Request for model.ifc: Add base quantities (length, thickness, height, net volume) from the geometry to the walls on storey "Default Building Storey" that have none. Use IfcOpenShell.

First a look at what the model holds.

```python
import ifcopenshell
import ifcopenshell.util.element
import ifcopenshell.util.unit

model = ifcopenshell.open("model.ifc")
print(model.schema)
for unit_type in ("LENGTHUNIT", "AREAUNIT", "VOLUMEUNIT"):
    print(unit_type, ifcopenshell.util.unit.calculate_unit_scale(model, unit_type))
storey = next(s for s in model.by_type("IfcBuildingStorey") if s.Name == "Default Building Storey")
walls = [e for e in ifcopenshell.util.element.get_decomposition(storey) if e.is_a("IfcWall")]
for e in sorted(walls, key=lambda e: e.id()):
    print(e.id(), e.is_a(), e.Name, list(ifcopenshell.util.element.get_psets(e, qtos_only=True)), sep=" | ")
```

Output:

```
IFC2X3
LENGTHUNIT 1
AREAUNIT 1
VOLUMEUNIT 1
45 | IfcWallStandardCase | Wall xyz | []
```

```python
import ifcopenshell
import ifcopenshell.api.pset
import ifcopenshell.geom
import ifcopenshell.util.element
import ifcopenshell.util.shape
import ifcopenshell.util.unit

model = ifcopenshell.open("model.ifc")
unit_scale = ifcopenshell.util.unit.calculate_unit_scale(model)
volume_scale = ifcopenshell.util.unit.calculate_unit_scale(model, "VOLUMEUNIT")
settings = ifcopenshell.geom.settings()

storey = next(s for s in model.by_type("IfcBuildingStorey") if s.Name == "Default Building Storey")
walls = [e for e in ifcopenshell.util.element.get_decomposition(storey) if e.is_a("IfcWall")]

for e in sorted(walls, key=lambda e: e.id()):
    if ifcopenshell.util.element.get_psets(e, qtos_only=True, should_inherit=False):
        continue
    # Geometry comes back in metres, in the element's own axes.
    shape = ifcopenshell.geom.create_shape(settings, e)
    values = {
        "Length": ifcopenshell.util.shape.get_x(shape.geometry) / unit_scale,
        "Width": ifcopenshell.util.shape.get_y(shape.geometry) / unit_scale,
        "Height": ifcopenshell.util.shape.get_z(shape.geometry) / unit_scale,
        "NetVolume": ifcopenshell.util.shape.get_volume(shape.geometry) / volume_scale,
    }
    qto = ifcopenshell.api.pset.add_qto(model, product=e, name="BaseQuantities")
    ifcopenshell.api.pset.edit_qto(model, qto=qto, properties=values)
    print(e.id(), {k: round(v, 3) for k, v in values.items()})

model.write("model_edited.ifc")
```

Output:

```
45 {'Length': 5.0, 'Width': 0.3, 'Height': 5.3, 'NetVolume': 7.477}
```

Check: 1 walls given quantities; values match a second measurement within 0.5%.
